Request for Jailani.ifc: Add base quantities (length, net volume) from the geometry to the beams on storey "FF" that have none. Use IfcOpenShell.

First a look at what the model holds.

```python
import ifcopenshell
import ifcopenshell.util.element
import ifcopenshell.util.unit

model = ifcopenshell.open("Jailani.ifc")
print(model.schema)
for unit_type in ("LENGTHUNIT", "AREAUNIT", "VOLUMEUNIT"):
    print(unit_type, ifcopenshell.util.unit.calculate_unit_scale(model, unit_type))
storey = next(s for s in model.by_type("IfcBuildingStorey") if s.Name == "FF")
beams = [e for e in ifcopenshell.util.element.get_decomposition(storey) if e.is_a("IfcBeam")]
for e in sorted(beams, key=lambda e: e.id()):
    print(e.id(), e.is_a(), e.Name, list(ifcopenshell.util.element.get_psets(e, qtos_only=True)), sep=" | ")
```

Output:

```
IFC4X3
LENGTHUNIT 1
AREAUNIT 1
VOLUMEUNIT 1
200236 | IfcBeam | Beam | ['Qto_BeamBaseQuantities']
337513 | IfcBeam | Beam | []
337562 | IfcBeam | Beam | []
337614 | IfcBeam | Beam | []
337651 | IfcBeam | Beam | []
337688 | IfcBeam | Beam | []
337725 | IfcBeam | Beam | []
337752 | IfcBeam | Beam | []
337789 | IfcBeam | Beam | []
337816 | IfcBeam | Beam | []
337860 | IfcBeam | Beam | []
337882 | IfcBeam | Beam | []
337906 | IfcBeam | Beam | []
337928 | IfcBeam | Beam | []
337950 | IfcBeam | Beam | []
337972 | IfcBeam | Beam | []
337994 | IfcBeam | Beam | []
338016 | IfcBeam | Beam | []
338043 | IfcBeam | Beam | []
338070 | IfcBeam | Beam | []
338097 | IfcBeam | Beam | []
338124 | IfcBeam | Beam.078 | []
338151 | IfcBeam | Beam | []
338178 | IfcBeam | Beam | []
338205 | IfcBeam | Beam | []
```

```python
import ifcopenshell
import ifcopenshell.api.pset
import ifcopenshell.geom
import ifcopenshell.util.element
import ifcopenshell.util.shape
import ifcopenshell.util.unit

model = ifcopenshell.open("Jailani.ifc")
unit_scale = ifcopenshell.util.unit.calculate_unit_scale(model)
volume_scale = ifcopenshell.util.unit.calculate_unit_scale(model, "VOLUMEUNIT")
settings = ifcopenshell.geom.settings()

storey = next(s for s in model.by_type("IfcBuildingStorey") if s.Name == "FF")
beams = [e for e in ifcopenshell.util.element.get_decomposition(storey) if e.is_a("IfcBeam")]

for e in sorted(beams, key=lambda e: e.id()):
    if ifcopenshell.util.element.get_psets(e, qtos_only=True, should_inherit=False):
        continue
    # Geometry comes back in metres, in the element's own axes.
    shape = ifcopenshell.geom.create_shape(settings, e)
    values = {
        "Length": ifcopenshell.util.shape.get_max_xyz(shape.geometry) / unit_scale,
        "NetVolume": ifcopenshell.util.shape.get_volume(shape.geometry) / volume_scale,
    }
    qto = ifcopenshell.api.pset.add_qto(model, product=e, name="Qto_BeamBaseQuantities")
    ifcopenshell.api.pset.edit_qto(model, qto=qto, properties=values)
    print(e.id(), {k: round(v, 3) for k, v in values.items()})

model.write("Jailani_rev.ifc")
```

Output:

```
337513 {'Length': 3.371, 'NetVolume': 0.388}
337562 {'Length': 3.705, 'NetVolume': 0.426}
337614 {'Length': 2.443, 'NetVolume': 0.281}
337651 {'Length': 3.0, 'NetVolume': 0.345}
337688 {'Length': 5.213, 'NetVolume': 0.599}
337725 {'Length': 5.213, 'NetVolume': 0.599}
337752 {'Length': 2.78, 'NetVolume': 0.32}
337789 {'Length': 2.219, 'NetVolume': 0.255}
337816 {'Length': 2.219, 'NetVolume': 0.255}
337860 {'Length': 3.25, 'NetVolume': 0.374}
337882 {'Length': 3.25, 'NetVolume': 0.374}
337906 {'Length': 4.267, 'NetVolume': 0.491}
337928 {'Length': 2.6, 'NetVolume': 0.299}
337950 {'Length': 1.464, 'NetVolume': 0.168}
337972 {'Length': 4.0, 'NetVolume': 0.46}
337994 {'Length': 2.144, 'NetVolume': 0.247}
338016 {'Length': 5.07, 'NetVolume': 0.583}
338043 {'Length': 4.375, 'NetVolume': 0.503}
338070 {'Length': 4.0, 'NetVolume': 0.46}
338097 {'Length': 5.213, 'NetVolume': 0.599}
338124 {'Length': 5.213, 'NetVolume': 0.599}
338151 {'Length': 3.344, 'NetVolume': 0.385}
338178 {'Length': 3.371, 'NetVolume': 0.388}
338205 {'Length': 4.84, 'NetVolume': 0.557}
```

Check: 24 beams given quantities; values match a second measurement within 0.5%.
